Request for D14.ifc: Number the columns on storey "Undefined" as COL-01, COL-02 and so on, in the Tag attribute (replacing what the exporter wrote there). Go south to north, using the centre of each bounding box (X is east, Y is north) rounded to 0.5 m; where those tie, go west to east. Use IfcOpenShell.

First a look at what the model holds.

```python
import ifcopenshell
import ifcopenshell.util.element
import ifcopenshell.util.placement

model = ifcopenshell.open("D14.ifc")
print(model.schema)
storey = next(s for s in model.by_type("IfcBuildingStorey") if s.Name == "Undefined")
columns = [e for e in ifcopenshell.util.element.get_decomposition(storey) if e.is_a("IfcColumn")]
for e in sorted(columns, key=lambda e: e.id()):
    origin = ifcopenshell.util.placement.get_local_placement(e.ObjectPlacement)[:3, 3]
    print(e.id(), e.Tag, e.Name, origin.round(2) + 0.0, sep=" | ")
```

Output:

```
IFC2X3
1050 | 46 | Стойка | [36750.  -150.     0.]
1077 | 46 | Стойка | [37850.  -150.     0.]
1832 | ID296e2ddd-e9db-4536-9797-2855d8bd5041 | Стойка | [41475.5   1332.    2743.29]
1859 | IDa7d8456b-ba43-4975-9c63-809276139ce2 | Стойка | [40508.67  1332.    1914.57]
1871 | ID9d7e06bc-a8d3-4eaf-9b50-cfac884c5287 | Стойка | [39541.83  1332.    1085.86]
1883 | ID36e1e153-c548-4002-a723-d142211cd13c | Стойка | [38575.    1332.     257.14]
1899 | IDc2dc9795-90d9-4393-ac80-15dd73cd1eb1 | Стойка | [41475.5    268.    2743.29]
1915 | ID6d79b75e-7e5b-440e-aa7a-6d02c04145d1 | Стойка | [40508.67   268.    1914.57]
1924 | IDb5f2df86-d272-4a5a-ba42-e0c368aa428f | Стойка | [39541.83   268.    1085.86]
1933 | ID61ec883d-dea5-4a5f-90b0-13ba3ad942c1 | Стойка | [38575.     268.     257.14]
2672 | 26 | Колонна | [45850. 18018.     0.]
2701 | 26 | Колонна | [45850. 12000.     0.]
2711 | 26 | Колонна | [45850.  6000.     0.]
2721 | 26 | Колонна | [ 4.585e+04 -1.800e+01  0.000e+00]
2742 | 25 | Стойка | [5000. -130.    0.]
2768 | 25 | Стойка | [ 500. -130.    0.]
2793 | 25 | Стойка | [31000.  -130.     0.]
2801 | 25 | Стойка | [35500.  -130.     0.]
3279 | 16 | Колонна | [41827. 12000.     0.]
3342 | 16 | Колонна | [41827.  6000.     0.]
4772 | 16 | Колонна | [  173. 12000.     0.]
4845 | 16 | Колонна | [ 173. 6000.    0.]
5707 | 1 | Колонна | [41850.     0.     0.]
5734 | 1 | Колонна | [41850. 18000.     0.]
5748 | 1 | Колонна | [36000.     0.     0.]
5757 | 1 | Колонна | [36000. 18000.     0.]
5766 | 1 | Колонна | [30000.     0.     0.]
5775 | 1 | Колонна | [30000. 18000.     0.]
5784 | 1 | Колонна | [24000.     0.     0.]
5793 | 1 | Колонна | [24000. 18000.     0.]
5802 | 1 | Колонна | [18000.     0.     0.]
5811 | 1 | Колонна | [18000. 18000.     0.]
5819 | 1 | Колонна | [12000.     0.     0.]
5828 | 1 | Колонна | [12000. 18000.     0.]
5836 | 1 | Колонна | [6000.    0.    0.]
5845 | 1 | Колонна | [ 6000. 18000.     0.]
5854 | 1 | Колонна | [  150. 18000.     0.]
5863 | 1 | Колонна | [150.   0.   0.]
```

```python
import ifcopenshell
import ifcopenshell.geom
import ifcopenshell.util.element
import ifcopenshell.util.shape

model = ifcopenshell.open("D14.ifc")
settings = ifcopenshell.geom.settings()
settings.set("use-world-coords", True)


def centre(element):
    shape = ifcopenshell.geom.create_shape(settings, element)
    return ifcopenshell.util.shape.get_bbox_centroid(shape.geometry)


storey = next(s for s in model.by_type("IfcBuildingStorey") if s.Name == "Undefined")
columns = [e for e in ifcopenshell.util.element.get_decomposition(storey) if e.is_a("IfcColumn")]

# Insertion points can sit at a corner or the storey origin, so sort by the geometry (in metres).
centres = {e: centre(e) for e in columns}
columns.sort(key=lambda e: (round(centres[e][1] / 0.5), centres[e][0]))

for i, e in enumerate(columns, start=1):
    number = f"COL-{i:02d}"
    e.Tag = number
    print(e.id(), number)

model.write("D14_rev.ifc")
```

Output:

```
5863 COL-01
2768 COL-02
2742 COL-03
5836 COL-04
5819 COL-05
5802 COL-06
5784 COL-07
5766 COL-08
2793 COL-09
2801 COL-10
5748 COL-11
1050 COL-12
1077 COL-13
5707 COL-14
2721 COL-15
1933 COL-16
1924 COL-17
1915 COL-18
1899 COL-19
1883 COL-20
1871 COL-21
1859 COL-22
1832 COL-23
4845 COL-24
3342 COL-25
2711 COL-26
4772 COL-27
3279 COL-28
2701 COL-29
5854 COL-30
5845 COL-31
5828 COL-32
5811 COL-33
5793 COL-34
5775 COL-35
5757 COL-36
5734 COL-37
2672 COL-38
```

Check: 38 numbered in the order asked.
